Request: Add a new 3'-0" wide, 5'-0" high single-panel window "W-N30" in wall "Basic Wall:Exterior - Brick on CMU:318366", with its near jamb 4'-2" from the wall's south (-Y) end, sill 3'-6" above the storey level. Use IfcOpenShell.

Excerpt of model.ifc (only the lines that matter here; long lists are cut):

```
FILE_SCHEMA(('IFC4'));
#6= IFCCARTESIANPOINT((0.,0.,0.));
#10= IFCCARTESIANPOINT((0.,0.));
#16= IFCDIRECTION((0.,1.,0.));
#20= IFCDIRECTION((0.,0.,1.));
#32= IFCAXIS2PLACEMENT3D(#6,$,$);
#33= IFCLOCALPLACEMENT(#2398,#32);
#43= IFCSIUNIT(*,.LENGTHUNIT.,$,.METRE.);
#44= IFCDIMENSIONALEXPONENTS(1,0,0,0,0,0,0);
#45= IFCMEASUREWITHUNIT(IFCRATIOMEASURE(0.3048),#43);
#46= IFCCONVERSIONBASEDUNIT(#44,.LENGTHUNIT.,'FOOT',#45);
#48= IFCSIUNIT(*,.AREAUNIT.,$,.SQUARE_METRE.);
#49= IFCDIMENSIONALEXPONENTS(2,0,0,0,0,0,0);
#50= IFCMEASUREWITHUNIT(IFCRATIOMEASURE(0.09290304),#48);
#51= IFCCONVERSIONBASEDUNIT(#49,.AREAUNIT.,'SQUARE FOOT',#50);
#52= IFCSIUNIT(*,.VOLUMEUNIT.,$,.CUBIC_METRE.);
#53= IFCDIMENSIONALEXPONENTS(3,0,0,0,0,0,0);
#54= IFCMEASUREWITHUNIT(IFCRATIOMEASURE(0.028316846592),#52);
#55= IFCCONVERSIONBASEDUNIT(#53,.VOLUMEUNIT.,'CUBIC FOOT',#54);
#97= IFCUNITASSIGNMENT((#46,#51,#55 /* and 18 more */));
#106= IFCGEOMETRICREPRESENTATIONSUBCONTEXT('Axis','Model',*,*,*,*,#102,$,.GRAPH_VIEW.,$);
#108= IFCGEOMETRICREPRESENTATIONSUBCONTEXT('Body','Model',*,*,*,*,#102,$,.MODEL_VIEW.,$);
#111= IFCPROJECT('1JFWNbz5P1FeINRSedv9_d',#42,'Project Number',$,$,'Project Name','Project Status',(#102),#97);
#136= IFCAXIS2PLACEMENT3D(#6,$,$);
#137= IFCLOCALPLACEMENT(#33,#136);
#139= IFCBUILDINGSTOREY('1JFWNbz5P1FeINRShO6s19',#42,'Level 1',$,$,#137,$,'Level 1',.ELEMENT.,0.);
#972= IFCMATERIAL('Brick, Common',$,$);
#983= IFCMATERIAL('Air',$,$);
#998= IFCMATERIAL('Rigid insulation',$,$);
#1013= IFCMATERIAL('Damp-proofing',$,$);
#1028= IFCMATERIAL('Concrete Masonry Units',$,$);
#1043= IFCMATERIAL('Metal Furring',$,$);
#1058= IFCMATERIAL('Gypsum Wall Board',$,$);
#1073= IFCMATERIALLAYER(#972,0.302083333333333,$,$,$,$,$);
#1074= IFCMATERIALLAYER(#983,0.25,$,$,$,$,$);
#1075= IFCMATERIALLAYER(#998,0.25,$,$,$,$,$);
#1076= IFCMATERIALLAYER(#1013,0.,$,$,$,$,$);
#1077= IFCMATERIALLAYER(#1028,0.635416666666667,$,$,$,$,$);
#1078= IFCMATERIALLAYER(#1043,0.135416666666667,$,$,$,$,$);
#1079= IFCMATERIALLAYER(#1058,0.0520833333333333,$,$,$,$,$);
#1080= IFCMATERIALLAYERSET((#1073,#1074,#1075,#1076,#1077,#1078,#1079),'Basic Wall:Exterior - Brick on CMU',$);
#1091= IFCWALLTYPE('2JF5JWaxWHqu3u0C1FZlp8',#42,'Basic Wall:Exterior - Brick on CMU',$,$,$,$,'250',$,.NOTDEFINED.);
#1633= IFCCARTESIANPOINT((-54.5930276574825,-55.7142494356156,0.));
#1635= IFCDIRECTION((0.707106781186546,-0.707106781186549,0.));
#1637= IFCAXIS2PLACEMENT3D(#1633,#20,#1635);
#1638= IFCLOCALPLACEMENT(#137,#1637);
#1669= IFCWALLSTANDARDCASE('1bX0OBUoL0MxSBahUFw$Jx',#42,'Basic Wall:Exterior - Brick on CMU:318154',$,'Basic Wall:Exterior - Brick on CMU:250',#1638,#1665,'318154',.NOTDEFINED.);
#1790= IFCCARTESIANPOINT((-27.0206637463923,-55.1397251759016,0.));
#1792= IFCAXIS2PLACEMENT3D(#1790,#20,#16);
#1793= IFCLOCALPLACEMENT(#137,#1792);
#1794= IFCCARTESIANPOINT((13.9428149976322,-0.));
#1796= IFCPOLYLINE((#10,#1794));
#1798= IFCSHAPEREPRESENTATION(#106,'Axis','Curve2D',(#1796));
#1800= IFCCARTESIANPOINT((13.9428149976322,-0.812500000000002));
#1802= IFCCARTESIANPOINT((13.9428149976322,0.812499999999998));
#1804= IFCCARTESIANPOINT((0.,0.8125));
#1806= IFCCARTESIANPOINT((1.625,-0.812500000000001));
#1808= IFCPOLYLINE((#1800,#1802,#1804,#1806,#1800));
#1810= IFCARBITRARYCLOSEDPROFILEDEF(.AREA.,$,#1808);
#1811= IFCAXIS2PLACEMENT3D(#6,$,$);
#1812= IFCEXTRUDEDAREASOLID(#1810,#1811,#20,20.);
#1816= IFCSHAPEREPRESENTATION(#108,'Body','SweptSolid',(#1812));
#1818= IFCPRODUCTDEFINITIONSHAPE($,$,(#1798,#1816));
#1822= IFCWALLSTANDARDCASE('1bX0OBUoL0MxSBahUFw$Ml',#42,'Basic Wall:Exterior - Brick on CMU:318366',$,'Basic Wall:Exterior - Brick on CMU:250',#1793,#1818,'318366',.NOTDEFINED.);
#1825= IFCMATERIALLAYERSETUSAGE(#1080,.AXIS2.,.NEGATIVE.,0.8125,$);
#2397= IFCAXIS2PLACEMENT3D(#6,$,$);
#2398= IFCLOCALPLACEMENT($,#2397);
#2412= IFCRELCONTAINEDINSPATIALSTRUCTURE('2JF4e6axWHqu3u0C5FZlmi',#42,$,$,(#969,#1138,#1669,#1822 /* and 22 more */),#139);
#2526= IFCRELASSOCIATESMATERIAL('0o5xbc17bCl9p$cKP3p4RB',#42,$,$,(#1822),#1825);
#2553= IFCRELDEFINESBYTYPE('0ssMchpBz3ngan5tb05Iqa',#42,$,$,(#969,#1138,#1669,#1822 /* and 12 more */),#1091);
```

```python
import numpy as np
import ifcopenshell
import ifcopenshell.api.feature
import ifcopenshell.api.geometry
import ifcopenshell.api.root
import ifcopenshell.api.spatial
import ifcopenshell.geom
import ifcopenshell.util.element
import ifcopenshell.util.placement
import ifcopenshell.util.representation
import ifcopenshell.util.shape
import ifcopenshell.util.unit

model = ifcopenshell.open("model.ifc")
unit_scale = ifcopenshell.util.unit.calculate_unit_scale(model)
settings = ifcopenshell.geom.settings()


def volume(element):
    """Net volume in cubic metres, openings subtracted."""
    shape = ifcopenshell.geom.create_shape(settings, element)
    return ifcopenshell.util.shape.get_volume(shape.geometry)


wall = model.by_guid("1bX0OBUoL0MxSBahUFw$Ml")
storey = ifcopenshell.util.element.get_container(wall, ifc_class="IfcBuildingStorey")
context = ifcopenshell.util.representation.get_context(model, "Model", "Body", "MODEL_VIEW")
before = volume(wall)

width, height, from_end, sill = 0.9144, 1.524, 1.27, 1.0668  # metres

# The wall runs along its own X axis, and the end named is its -X end.
wall_shape = ifcopenshell.geom.create_shape(settings, wall)
x, y, z = ifcopenshell.util.shape.get_vertices(wall_shape.geometry).T
start = x.min() + from_end
face, thickness = float(y.min()), float(y.max() - y.min())
wall_matrix = ifcopenshell.util.placement.get_local_placement(wall.ObjectPlacement)
level = ifcopenshell.util.placement.get_local_placement(storey.ObjectPlacement)[2, 3]


def in_wall(x, y):
    """Placement at x, y metres in the wall's axes, at sill height."""
    matrix = wall_matrix.copy()
    matrix[:, 3] = wall_matrix @ np.array([x / unit_scale, y / unit_scale, 0.0, 1.0])
    matrix[2, 3] = level + sill / unit_scale
    return matrix


# Opening: a box that overshoots both wall faces by 50 mm.
opening = ifcopenshell.api.root.create_entity(model, ifc_class="IfcOpeningElement", predefined_type="OPENING")
box = ifcopenshell.api.geometry.add_wall_representation(
    model, context=context, length=width, height=height, thickness=thickness + 0.1
)
ifcopenshell.api.geometry.assign_representation(model, product=opening, representation=box)
ifcopenshell.api.geometry.edit_object_placement(model, product=opening, matrix=in_wall(start, face - 0.05), is_si=False)
ifcopenshell.api.feature.add_feature(model, feature=opening, element=wall)

window = ifcopenshell.api.root.create_entity(model, ifc_class="IfcWindow", name="W-N30", predefined_type="WINDOW")
window.OverallWidth, window.OverallHeight = width / unit_scale, height / unit_scale
window.PartitioningType = "SINGLE_PANEL"
body = ifcopenshell.api.geometry.add_window_representation(
    model,
    context=context,
    overall_width=window.OverallWidth,
    overall_height=window.OverallHeight,
    partition_type="SINGLE_PANEL",
)
ifcopenshell.api.geometry.assign_representation(model, product=window, representation=body)
ifcopenshell.api.spatial.assign_container(model, products=[window], relating_structure=storey)
ifcopenshell.api.feature.add_filling(model, opening=opening, element=window)

# Centre the window in the wall's thickness.
ifcopenshell.api.geometry.edit_object_placement(model, product=window, matrix=in_wall(start, face), is_si=False)
window_shape = ifcopenshell.geom.create_shape(settings, window)
depth = ifcopenshell.util.shape.get_vertices(window_shape.geometry)[:, 1]
offset = face + thickness / 2 - (depth.min() + depth.max()) / 2
ifcopenshell.api.geometry.edit_object_placement(model, product=window, matrix=in_wall(start, offset), is_si=False)

after = volume(wall)

print(f"wall volume {before:.3f} -> {after:.3f} m3")

model.write("model_v2.ifc")
```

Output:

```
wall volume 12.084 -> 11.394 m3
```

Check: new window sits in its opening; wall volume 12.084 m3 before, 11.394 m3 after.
